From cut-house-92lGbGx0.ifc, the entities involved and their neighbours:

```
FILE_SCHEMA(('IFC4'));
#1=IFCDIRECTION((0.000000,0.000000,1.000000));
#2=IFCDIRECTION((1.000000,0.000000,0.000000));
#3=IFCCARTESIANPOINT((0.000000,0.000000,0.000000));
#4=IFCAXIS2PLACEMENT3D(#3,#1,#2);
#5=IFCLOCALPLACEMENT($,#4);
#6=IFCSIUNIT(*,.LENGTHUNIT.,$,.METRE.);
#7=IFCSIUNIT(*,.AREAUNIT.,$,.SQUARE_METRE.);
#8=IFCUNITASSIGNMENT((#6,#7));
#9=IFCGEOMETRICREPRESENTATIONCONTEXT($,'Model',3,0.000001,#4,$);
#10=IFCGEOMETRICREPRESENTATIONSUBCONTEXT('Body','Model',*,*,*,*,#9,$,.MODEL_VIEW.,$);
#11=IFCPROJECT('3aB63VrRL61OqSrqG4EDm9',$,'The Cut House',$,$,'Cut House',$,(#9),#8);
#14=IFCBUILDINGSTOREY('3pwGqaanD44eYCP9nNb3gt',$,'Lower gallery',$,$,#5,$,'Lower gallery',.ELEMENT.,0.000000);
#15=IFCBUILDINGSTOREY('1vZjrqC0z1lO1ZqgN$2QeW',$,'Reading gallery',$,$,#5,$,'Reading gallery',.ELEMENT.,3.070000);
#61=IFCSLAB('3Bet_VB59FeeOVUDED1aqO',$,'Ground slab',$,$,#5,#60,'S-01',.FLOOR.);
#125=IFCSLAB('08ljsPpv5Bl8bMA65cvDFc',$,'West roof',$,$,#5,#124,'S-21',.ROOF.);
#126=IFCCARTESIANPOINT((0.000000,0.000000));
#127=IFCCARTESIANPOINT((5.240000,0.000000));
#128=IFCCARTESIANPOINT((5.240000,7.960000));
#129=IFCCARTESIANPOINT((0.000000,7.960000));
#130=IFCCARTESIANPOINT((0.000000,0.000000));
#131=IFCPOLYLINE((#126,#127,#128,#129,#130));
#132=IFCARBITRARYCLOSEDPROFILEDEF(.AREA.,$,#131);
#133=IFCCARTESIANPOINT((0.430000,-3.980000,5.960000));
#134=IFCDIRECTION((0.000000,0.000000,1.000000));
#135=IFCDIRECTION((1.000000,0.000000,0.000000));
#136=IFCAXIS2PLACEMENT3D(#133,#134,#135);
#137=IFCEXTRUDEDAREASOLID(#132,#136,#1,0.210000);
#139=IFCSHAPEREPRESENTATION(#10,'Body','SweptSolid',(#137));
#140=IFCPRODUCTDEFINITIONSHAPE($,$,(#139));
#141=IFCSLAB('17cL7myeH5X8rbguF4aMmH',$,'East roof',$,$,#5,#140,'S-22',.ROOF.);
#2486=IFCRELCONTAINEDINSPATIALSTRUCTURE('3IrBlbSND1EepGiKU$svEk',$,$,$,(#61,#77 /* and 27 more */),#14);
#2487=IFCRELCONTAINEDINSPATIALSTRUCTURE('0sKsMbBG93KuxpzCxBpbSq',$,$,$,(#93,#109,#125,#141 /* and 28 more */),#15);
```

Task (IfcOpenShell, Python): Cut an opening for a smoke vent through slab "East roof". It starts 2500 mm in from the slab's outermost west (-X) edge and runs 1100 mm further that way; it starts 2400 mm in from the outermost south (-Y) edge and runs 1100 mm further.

```python
import numpy as np
import ifcopenshell
import ifcopenshell.api.feature
import ifcopenshell.api.geometry
import ifcopenshell.api.root
import ifcopenshell.geom
import ifcopenshell.util.placement
import ifcopenshell.util.representation
import ifcopenshell.util.shape
import ifcopenshell.util.unit

model = ifcopenshell.open("cut-house-92lGbGx0.ifc")
unit_scale = ifcopenshell.util.unit.calculate_unit_scale(model)
settings = ifcopenshell.geom.settings()


def volume(element):
    """Net volume in cubic metres, openings subtracted."""
    shape = ifcopenshell.geom.create_shape(settings, element)
    return ifcopenshell.util.shape.get_volume(shape.geometry)


slab = model.by_guid("17cL7myeH5X8rbguF4aMmH")
before = volume(slab)

# Extent in the slab's own axes, in metres. The edges named are its -X and -Y sides.
slab_shape = ifcopenshell.geom.create_shape(settings, slab)
vertices = ifcopenshell.util.shape.get_vertices(slab_shape.geometry)
x_min, y_min, bottom = vertices.min(axis=0)
top = vertices[:, 2].max()

opening = ifcopenshell.api.root.create_entity(model, ifc_class="IfcOpeningElement", name="Smoke vent opening", predefined_type="OPENING")
context = ifcopenshell.util.representation.get_context(model, "Model", "Body", "MODEL_VIEW")
width, depth = 1.1, 1.1
outline = [(0.0, 0.0), (width, 0.0), (width, depth), (0.0, depth), (0.0, 0.0)]
# Overshoot both faces by 50 mm so the cut is clean.
shape = ifcopenshell.api.geometry.add_slab_representation(
    model, context=context, depth=top - bottom + 0.1, polyline=outline
)
ifcopenshell.api.geometry.assign_representation(model, product=opening, representation=shape)

matrix = ifcopenshell.util.placement.get_local_placement(slab.ObjectPlacement)
matrix[:, 3] = matrix @ np.append(np.array([x_min + 2.5, y_min + 2.4, bottom - 0.05]) / unit_scale, 1.0)
ifcopenshell.api.geometry.edit_object_placement(model, product=opening, matrix=matrix, is_si=False)
ifcopenshell.api.feature.add_feature(model, feature=opening, element=slab)

after = volume(slab)

print(f"slab volume {before:.3f} -> {after:.3f} m3")

model.write("cut-house-92lGbGx0-out.ifc")
```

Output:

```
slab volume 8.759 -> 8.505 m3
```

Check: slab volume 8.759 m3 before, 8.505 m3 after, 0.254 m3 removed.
